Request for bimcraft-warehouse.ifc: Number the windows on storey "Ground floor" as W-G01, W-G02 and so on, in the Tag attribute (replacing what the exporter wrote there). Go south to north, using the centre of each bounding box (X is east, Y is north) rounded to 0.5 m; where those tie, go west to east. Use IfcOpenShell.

First a look at what the model holds.

```python
import ifcopenshell
import ifcopenshell.util.element
import ifcopenshell.util.placement

model = ifcopenshell.open("bimcraft-warehouse.ifc")
print(model.schema)
storey = next(s for s in model.by_type("IfcBuildingStorey") if s.Name == "Ground floor")
windows = [e for e in ifcopenshell.util.element.get_decomposition(storey) if e.is_a("IfcWindow")]
for e in sorted(windows, key=lambda e: e.id()):
    origin = ifcopenshell.util.placement.get_local_placement(e.ObjectPlacement)[:3, 3]
    print(e.id(), e.Tag, e.Name, origin.round(2) + 0.0, sep=" | ")
```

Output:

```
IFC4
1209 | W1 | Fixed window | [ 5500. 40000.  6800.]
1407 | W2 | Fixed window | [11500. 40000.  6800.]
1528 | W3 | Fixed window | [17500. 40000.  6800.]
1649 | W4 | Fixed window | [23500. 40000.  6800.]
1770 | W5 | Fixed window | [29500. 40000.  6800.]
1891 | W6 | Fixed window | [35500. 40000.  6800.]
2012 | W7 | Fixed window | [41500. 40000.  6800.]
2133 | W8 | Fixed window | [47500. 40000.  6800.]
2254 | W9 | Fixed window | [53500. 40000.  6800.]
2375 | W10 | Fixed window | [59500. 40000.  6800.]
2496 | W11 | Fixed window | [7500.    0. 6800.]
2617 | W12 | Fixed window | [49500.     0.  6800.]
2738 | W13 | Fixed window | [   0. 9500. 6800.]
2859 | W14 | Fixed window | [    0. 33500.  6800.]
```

```python
import ifcopenshell
import ifcopenshell.geom
import ifcopenshell.util.element
import ifcopenshell.util.shape

model = ifcopenshell.open("bimcraft-warehouse.ifc")
settings = ifcopenshell.geom.settings()
settings.set("use-world-coords", True)


def centre(element):
    shape = ifcopenshell.geom.create_shape(settings, element)
    return ifcopenshell.util.shape.get_bbox_centroid(shape.geometry)


storey = next(s for s in model.by_type("IfcBuildingStorey") if s.Name == "Ground floor")
windows = [e for e in ifcopenshell.util.element.get_decomposition(storey) if e.is_a("IfcWindow")]

# Insertion points can sit at a corner or the storey origin, so sort by the geometry (in metres).
centres = {e: centre(e) for e in windows}
windows.sort(key=lambda e: (round(centres[e][1] / 0.5), centres[e][0]))

for i, e in enumerate(windows, start=1):
    number = f"W-G{i:02d}"
    e.Tag = number
    print(e.id(), number)

model.write("bimcraft-warehouse_updated.ifc")
```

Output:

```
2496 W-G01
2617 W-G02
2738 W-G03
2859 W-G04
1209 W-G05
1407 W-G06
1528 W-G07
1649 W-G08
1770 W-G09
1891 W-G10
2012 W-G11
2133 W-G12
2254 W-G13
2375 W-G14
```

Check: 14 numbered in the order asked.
